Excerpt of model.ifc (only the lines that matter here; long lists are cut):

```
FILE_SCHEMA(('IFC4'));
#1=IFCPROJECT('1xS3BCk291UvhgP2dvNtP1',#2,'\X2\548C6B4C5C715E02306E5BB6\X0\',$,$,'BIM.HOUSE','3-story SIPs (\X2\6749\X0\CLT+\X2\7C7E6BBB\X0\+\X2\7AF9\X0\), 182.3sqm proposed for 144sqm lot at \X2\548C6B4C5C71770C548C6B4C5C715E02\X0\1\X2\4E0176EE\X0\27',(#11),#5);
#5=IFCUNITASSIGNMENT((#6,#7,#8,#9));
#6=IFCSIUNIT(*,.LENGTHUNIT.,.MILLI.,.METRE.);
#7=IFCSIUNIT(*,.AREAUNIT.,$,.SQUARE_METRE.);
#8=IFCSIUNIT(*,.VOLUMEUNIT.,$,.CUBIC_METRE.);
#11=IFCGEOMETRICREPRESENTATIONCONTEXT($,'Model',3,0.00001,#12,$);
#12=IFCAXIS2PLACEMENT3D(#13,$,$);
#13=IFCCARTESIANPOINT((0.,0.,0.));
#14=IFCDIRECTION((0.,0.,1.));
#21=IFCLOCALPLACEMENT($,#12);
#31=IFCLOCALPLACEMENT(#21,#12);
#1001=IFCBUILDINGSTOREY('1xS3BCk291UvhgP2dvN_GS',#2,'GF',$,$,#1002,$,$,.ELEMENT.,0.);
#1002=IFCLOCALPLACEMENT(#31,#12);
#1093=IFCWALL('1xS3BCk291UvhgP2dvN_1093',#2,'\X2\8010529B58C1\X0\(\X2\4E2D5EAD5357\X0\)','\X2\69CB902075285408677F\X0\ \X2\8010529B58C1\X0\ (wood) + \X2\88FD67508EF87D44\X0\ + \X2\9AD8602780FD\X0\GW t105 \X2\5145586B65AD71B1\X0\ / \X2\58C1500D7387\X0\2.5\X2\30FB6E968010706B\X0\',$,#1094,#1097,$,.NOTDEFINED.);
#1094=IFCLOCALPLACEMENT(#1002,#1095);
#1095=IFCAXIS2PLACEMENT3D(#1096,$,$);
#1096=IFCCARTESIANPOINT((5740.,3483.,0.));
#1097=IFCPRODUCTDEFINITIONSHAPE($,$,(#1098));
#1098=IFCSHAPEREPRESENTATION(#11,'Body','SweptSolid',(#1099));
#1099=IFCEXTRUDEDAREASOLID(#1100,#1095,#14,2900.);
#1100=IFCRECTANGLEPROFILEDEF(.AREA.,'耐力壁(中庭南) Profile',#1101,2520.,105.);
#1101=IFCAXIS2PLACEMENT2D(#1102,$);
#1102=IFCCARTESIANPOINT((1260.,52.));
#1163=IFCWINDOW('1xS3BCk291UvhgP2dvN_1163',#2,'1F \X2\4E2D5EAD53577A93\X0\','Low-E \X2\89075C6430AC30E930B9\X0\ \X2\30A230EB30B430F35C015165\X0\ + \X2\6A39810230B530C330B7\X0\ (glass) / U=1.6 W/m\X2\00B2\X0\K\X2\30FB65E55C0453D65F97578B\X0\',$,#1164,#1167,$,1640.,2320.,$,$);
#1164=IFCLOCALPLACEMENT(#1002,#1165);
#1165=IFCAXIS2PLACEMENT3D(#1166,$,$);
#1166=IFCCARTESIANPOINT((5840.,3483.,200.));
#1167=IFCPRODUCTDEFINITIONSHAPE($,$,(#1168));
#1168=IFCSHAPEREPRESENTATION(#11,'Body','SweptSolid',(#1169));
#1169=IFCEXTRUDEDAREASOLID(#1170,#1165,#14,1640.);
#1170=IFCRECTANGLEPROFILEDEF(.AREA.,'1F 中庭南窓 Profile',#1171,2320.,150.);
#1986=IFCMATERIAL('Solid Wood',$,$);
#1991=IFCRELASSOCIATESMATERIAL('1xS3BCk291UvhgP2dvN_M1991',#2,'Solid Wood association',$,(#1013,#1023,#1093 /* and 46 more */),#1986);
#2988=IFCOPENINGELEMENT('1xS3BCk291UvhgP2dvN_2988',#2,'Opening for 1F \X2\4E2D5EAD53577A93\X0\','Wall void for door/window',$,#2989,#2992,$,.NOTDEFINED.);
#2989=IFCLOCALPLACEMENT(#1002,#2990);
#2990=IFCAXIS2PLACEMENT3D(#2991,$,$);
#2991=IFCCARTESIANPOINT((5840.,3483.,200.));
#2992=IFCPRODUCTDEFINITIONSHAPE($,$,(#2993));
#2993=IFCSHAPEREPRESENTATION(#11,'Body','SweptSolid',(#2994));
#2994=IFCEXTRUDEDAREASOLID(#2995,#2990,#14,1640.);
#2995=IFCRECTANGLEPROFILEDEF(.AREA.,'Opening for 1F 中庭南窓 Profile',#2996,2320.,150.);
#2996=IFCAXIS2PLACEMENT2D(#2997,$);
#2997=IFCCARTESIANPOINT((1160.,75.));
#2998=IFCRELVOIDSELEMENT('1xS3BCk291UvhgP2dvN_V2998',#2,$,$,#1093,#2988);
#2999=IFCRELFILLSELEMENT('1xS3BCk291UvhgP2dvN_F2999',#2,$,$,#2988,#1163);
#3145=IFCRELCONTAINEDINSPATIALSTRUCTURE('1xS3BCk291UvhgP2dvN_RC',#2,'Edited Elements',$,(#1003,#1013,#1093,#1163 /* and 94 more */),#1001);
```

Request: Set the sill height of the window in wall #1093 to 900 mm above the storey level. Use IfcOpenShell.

```python
import numpy as np
import ifcopenshell
import ifcopenshell.api.geometry
import ifcopenshell.geom
import ifcopenshell.util.element
import ifcopenshell.util.placement
import ifcopenshell.util.shape
import ifcopenshell.util.unit

model = ifcopenshell.open("model.ifc")
unit_scale = ifcopenshell.util.unit.calculate_unit_scale(model)

window = model.by_guid("1xS3BCk291UvhgP2dvN_1163")
opening = window.FillsVoids[0].RelatingOpeningElement
storey = ifcopenshell.util.element.get_container(window, ifc_class="IfcBuildingStorey")
level = ifcopenshell.util.placement.get_local_placement(storey.ObjectPlacement)[2, 3]

# The opening's origin need not be at the sill, so measure its lowest point.
shape = ifcopenshell.geom.create_shape(ifcopenshell.geom.settings(), opening)
bottom = ifcopenshell.util.shape.get_shape_bottom_elevation(shape, shape.geometry) / unit_scale
dz = level + 900.0 - bottom

shift = np.array([0.0, 0.0, dz])
# The window is not placed relative to its opening, so move both.
for product in (opening, window):
    matrix = ifcopenshell.util.placement.get_local_placement(product.ObjectPlacement)
    matrix[:3, 3] += shift
    ifcopenshell.api.geometry.edit_object_placement(model, product=product, matrix=matrix, is_si=False)

print(f"moved by {dz * unit_scale:+.3f} m")

model.write("model-out.ifc")
```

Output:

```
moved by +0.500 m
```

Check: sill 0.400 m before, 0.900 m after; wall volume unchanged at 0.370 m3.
